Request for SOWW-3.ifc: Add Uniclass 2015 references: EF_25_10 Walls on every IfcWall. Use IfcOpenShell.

First a look at what the model holds.

```python
import ifcopenshell

model = ifcopenshell.open("SOWW-3.ifc")
print(model.schema)
print("classifications:", [c.Name for c in model.by_type("IfcClassification")])
for ifc_class in ("IfcDoor", "IfcRoof", "IfcStair", "IfcWall", "IfcWindow"):
    print(ifc_class, len(model.by_type(ifc_class)))
```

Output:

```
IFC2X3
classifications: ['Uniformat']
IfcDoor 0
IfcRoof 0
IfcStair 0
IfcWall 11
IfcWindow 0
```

```python
import ifcopenshell
import ifcopenshell.api.classification

model = ifcopenshell.open("SOWW-3.ifc")

# IFC2X3 requires Source and Edition and has no link from the project to the system.
system = model.create_entity("IfcClassification", Source="NBS", Edition="2015", Name="Uniclass 2015")

codes = {
    "IfcWall": ("EF_25_10", "Walls"),
}
for ifc_class, (code, name) in codes.items():
    products = model.by_type(ifc_class)
    ifcopenshell.api.classification.add_reference(
        model, products=products, classification=system, identification=code, name=name
    )
    print(code, len(products))

model.write("SOWW-3_updated.ifc")
```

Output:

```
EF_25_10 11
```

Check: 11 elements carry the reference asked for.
